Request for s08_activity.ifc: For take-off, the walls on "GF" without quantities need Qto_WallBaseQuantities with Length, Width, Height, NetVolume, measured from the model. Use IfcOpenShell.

First a look at what the model holds.

```python
import ifcopenshell
import ifcopenshell.util.element
import ifcopenshell.util.unit

model = ifcopenshell.open("s08_activity.ifc")
print(model.schema)
for unit_type in ("LENGTHUNIT", "AREAUNIT", "VOLUMEUNIT"):
    print(unit_type, ifcopenshell.util.unit.calculate_unit_scale(model, unit_type))
storey = next(s for s in model.by_type("IfcBuildingStorey") if s.Name == "GF")
walls = [e for e in ifcopenshell.util.element.get_decomposition(storey) if e.is_a("IfcWall")]
for e in sorted(walls, key=lambda e: e.id()):
    print(e.id(), e.is_a(), e.Name, list(ifcopenshell.util.element.get_psets(e, qtos_only=True)), sep=" | ")
```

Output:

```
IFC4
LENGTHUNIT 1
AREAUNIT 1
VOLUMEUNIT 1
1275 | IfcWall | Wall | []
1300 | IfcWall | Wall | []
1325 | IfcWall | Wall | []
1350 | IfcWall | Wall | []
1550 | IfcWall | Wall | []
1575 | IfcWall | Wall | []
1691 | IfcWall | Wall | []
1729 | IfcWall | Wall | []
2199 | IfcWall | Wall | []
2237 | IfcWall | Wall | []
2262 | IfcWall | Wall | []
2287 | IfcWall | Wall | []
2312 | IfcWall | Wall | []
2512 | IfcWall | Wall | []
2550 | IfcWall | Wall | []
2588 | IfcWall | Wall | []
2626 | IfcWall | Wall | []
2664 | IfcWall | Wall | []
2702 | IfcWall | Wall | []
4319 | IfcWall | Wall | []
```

```python
import ifcopenshell
import ifcopenshell.api.pset
import ifcopenshell.geom
import ifcopenshell.util.element
import ifcopenshell.util.shape
import ifcopenshell.util.unit

model = ifcopenshell.open("s08_activity.ifc")
unit_scale = ifcopenshell.util.unit.calculate_unit_scale(model)
volume_scale = ifcopenshell.util.unit.calculate_unit_scale(model, "VOLUMEUNIT")
settings = ifcopenshell.geom.settings()

storey = next(s for s in model.by_type("IfcBuildingStorey") if s.Name == "GF")
walls = [e for e in ifcopenshell.util.element.get_decomposition(storey) if e.is_a("IfcWall")]

for e in sorted(walls, key=lambda e: e.id()):
    if ifcopenshell.util.element.get_psets(e, qtos_only=True, should_inherit=False):
        continue
    # Geometry comes back in metres, in the element's own axes.
    shape = ifcopenshell.geom.create_shape(settings, e)
    values = {
        "Length": ifcopenshell.util.shape.get_x(shape.geometry) / unit_scale,
        "Width": ifcopenshell.util.shape.get_y(shape.geometry) / unit_scale,
        "Height": ifcopenshell.util.shape.get_z(shape.geometry) / unit_scale,
        "NetVolume": ifcopenshell.util.shape.get_volume(shape.geometry) / volume_scale,
    }
    qto = ifcopenshell.api.pset.add_qto(model, product=e, name="Qto_WallBaseQuantities")
    ifcopenshell.api.pset.edit_qto(model, qto=qto, properties=values)
    print(e.id(), {k: round(v, 3) for k, v in values.items()})

model.write("s08_activity_updated.ifc")
```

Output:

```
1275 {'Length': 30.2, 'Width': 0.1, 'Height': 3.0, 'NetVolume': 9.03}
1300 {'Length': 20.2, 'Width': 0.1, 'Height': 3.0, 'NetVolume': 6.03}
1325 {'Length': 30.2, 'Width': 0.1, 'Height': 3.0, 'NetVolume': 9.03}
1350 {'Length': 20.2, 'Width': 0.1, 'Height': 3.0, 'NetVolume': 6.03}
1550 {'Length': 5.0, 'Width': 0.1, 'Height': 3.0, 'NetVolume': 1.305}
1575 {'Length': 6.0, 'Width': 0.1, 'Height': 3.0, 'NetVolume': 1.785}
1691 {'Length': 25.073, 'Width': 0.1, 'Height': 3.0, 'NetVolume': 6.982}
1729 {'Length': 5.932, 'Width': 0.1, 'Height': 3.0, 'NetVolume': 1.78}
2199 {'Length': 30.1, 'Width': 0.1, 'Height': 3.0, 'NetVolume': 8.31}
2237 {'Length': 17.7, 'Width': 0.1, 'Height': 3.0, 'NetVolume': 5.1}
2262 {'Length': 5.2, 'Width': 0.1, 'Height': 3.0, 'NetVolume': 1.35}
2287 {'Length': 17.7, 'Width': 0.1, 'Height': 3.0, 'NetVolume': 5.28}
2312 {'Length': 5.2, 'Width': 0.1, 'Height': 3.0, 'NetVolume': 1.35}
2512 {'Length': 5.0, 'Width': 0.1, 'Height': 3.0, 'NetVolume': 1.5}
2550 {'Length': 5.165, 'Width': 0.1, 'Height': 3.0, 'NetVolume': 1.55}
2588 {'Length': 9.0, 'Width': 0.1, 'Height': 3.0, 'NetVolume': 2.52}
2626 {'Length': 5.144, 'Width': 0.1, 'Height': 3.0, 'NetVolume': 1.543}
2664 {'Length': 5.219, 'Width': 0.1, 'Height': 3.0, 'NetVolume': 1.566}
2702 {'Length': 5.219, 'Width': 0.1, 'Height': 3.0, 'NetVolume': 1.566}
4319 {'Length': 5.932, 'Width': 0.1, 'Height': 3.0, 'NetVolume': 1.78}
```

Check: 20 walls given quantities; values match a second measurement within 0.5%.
